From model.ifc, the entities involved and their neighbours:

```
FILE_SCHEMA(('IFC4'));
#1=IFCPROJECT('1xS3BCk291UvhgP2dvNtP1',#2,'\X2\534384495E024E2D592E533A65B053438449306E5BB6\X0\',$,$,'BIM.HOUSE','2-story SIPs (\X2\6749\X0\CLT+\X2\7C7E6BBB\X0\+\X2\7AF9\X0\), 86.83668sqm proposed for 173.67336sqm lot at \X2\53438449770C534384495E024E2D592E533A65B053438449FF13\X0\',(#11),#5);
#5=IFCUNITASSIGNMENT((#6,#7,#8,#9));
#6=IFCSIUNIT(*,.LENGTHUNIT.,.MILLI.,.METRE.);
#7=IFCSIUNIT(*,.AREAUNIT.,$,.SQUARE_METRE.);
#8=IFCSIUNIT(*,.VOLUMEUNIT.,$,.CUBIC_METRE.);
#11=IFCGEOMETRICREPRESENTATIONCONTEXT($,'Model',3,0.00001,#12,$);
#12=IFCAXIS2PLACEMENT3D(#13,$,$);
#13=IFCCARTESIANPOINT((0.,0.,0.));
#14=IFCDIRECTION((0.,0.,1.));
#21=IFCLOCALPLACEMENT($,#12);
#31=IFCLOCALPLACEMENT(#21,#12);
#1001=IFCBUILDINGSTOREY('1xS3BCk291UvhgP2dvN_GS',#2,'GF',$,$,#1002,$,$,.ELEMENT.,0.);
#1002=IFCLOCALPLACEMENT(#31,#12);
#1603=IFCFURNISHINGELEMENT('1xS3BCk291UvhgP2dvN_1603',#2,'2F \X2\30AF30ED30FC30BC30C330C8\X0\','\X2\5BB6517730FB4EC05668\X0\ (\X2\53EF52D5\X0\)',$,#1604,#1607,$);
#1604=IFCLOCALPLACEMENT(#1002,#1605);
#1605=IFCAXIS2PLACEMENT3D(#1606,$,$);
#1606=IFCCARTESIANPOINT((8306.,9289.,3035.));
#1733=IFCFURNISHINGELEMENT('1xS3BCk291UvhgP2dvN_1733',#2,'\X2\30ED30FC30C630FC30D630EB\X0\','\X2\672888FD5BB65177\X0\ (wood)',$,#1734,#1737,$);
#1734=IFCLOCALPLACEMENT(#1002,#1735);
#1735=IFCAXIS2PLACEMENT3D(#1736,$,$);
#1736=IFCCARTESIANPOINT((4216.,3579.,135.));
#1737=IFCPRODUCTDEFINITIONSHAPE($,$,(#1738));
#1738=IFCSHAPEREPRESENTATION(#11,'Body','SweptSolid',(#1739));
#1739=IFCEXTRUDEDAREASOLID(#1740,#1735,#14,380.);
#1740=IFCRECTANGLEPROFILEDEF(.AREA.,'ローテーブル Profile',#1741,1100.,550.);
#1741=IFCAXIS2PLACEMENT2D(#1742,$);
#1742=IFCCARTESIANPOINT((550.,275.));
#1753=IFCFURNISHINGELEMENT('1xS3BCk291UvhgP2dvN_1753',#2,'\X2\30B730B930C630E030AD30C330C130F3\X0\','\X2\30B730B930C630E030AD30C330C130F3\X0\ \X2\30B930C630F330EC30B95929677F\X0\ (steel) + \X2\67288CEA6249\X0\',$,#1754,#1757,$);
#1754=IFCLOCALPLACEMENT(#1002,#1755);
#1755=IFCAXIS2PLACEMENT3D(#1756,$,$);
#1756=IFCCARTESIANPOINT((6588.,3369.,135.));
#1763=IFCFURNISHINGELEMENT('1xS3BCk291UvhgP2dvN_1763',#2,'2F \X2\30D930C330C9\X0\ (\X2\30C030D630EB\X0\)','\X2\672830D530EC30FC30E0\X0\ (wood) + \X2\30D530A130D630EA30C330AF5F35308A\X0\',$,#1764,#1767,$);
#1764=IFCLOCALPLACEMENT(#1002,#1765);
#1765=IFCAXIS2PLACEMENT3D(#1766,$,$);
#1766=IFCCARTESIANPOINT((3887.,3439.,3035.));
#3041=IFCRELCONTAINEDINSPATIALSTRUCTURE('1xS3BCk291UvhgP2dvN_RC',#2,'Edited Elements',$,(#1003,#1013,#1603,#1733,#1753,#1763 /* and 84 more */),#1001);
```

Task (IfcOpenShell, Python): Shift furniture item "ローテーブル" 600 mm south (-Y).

```python
import ifcopenshell
import ifcopenshell.api.geometry
import ifcopenshell.util.placement

model = ifcopenshell.open("model.ifc")

item = model.by_id(1733)
matrix = ifcopenshell.util.placement.get_local_placement(item.ObjectPlacement)
matrix[1, 3] -= 600.0
ifcopenshell.api.geometry.edit_object_placement(model, product=item, matrix=matrix, is_si=False)

print(ifcopenshell.util.placement.get_local_placement(item.ObjectPlacement).round(3) + 0.0)

model.write("model_rev.ifc")
```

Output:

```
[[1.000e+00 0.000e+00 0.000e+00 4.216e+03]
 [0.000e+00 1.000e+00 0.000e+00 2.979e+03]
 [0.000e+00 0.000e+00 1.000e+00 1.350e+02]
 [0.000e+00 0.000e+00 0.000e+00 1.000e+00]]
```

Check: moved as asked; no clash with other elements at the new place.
